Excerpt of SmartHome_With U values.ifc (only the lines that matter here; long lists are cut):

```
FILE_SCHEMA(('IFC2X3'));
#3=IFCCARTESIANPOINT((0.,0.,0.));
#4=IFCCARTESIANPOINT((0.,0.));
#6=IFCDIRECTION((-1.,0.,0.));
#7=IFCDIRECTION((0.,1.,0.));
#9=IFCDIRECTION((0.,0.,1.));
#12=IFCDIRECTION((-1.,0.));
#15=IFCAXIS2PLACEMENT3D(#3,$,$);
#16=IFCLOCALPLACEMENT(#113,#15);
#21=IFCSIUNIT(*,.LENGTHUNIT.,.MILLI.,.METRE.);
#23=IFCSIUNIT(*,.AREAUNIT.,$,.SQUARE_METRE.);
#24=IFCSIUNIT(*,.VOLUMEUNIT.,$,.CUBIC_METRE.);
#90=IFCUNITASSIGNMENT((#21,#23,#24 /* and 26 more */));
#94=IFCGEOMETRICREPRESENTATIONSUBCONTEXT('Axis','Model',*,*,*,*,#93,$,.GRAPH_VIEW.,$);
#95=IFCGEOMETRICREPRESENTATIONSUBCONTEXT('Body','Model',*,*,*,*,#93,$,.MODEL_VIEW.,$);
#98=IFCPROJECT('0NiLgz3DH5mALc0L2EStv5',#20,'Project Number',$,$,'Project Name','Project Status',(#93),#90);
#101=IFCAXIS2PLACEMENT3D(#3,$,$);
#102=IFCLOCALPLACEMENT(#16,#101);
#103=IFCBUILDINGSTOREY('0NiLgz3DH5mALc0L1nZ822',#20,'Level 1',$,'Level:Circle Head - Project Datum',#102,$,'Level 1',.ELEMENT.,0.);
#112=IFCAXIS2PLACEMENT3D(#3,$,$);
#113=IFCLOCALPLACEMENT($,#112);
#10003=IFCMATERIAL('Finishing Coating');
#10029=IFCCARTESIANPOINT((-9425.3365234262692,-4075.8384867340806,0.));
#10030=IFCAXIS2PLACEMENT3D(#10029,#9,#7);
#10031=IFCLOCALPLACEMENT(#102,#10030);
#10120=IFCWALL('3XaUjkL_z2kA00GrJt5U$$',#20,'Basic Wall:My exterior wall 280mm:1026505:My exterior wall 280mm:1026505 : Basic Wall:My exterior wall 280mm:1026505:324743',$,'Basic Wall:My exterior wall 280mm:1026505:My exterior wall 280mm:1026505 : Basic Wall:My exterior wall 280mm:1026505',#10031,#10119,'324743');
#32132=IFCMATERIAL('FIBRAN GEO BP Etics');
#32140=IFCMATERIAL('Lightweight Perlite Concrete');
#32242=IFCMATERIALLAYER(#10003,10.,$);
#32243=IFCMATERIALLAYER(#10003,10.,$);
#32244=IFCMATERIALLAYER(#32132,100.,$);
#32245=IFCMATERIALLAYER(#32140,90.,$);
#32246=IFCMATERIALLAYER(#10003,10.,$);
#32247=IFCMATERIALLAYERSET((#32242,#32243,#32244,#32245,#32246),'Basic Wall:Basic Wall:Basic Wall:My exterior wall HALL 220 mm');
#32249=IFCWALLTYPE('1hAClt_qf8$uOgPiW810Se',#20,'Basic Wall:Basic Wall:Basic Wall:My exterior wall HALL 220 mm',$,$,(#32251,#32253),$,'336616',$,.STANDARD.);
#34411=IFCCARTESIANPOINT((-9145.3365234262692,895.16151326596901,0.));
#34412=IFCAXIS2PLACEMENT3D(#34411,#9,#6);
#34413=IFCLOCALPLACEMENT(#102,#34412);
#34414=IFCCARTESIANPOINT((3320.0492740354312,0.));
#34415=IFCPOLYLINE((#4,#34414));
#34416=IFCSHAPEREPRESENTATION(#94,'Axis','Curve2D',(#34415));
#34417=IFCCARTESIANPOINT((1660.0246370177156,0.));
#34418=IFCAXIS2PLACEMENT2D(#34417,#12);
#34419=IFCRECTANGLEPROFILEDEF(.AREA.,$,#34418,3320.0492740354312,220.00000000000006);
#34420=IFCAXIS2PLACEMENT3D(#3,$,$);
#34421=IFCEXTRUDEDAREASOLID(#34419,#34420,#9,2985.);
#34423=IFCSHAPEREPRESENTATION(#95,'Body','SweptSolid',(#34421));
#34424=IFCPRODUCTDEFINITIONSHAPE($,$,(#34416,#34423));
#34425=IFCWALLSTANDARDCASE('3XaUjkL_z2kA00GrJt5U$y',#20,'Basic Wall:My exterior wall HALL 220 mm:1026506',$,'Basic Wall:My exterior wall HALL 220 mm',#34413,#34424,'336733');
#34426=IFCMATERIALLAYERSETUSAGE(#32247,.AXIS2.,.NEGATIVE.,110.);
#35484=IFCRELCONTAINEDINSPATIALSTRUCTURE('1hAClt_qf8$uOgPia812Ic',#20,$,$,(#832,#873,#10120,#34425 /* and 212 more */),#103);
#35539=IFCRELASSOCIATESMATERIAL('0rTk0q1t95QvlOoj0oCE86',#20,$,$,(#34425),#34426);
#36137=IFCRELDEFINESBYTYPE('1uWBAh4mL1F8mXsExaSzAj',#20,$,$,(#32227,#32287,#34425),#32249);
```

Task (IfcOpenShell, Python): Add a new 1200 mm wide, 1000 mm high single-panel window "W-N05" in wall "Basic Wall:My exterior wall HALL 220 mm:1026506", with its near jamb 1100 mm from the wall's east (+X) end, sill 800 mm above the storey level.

```python
import numpy as np
import ifcopenshell
import ifcopenshell.api.feature
import ifcopenshell.api.geometry
import ifcopenshell.api.root
import ifcopenshell.api.spatial
import ifcopenshell.api.type
import ifcopenshell.geom
import ifcopenshell.util.element
import ifcopenshell.util.placement
import ifcopenshell.util.representation
import ifcopenshell.util.shape
import ifcopenshell.util.unit

model = ifcopenshell.open("SmartHome_With U values.ifc")
unit_scale = ifcopenshell.util.unit.calculate_unit_scale(model)
settings = ifcopenshell.geom.settings()


def volume(element):
    """Net volume in cubic metres, openings subtracted."""
    shape = ifcopenshell.geom.create_shape(settings, element)
    return ifcopenshell.util.shape.get_volume(shape.geometry)


wall = model.by_guid("3XaUjkL_z2kA00GrJt5U$y")
storey = ifcopenshell.util.element.get_container(wall, ifc_class="IfcBuildingStorey")
context = ifcopenshell.util.representation.get_context(model, "Model", "Body", "MODEL_VIEW")
before = volume(wall)

width, height, from_end, sill = 1.2, 1, 1.1, 0.8  # metres

# The wall runs along its own X axis, and the end named is its -X end.
wall_shape = ifcopenshell.geom.create_shape(settings, wall)
x, y, z = ifcopenshell.util.shape.get_vertices(wall_shape.geometry).T
start = x.min() + from_end
face, thickness = float(y.min()), float(y.max() - y.min())
wall_matrix = ifcopenshell.util.placement.get_local_placement(wall.ObjectPlacement)
level = ifcopenshell.util.placement.get_local_placement(storey.ObjectPlacement)[2, 3]


def in_wall(x, y):
    """Placement at x, y metres in the wall's axes, at sill height."""
    matrix = wall_matrix.copy()
    matrix[:, 3] = wall_matrix @ np.array([x / unit_scale, y / unit_scale, 0.0, 1.0])
    matrix[2, 3] = level + sill / unit_scale
    return matrix


# Opening: a box that overshoots both wall faces by 50 mm.
opening = ifcopenshell.api.root.create_entity(model, ifc_class="IfcOpeningElement")
box = ifcopenshell.api.geometry.add_wall_representation(
    model, context=context, length=width, height=height, thickness=thickness + 0.1
)
ifcopenshell.api.geometry.assign_representation(model, product=opening, representation=box)
ifcopenshell.api.geometry.edit_object_placement(model, product=opening, matrix=in_wall(start, face - 0.05), is_si=False)
ifcopenshell.api.feature.add_feature(model, feature=opening, element=wall)

window = ifcopenshell.api.root.create_entity(model, ifc_class="IfcWindow", name="W-N05")
window.OverallWidth, window.OverallHeight = width / unit_scale, height / unit_scale
body = ifcopenshell.api.geometry.add_window_representation(
    model,
    context=context,
    overall_width=window.OverallWidth,
    overall_height=window.OverallHeight,
    partition_type="SINGLE_PANEL",
)
ifcopenshell.api.geometry.assign_representation(model, product=window, representation=body)
ifcopenshell.api.spatial.assign_container(model, products=[window], relating_structure=storey)
fills = ifcopenshell.api.feature.add_filling(model, opening=opening, element=window)
fills.OwnerHistory = window.OwnerHistory  # required in IFC2X3

# IFC2X3 keeps the operation on the window style.
style = ifcopenshell.api.root.create_entity(model, ifc_class="IfcWindowStyle", name="W-N05")
style.OperationType, style.ConstructionType = "SINGLE_PANEL", "NOTDEFINED"
style.ParameterTakesPrecedence = style.Sizeable = False
ifcopenshell.api.type.assign_type(model, related_objects=[window], relating_type=style)

# Centre the window in the wall's thickness.
ifcopenshell.api.geometry.edit_object_placement(model, product=window, matrix=in_wall(start, face), is_si=False)
window_shape = ifcopenshell.geom.create_shape(settings, window)
depth = ifcopenshell.util.shape.get_vertices(window_shape.geometry)[:, 1]
offset = face + thickness / 2 - (depth.min() + depth.max()) / 2
ifcopenshell.api.geometry.edit_object_placement(model, product=window, matrix=in_wall(start, offset), is_si=False)

after = volume(wall)

print(f"wall volume {before:.3f} -> {after:.3f} m3")

model.write("SmartHome_With U values-out.ifc")
```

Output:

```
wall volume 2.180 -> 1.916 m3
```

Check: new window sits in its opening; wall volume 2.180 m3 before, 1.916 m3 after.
